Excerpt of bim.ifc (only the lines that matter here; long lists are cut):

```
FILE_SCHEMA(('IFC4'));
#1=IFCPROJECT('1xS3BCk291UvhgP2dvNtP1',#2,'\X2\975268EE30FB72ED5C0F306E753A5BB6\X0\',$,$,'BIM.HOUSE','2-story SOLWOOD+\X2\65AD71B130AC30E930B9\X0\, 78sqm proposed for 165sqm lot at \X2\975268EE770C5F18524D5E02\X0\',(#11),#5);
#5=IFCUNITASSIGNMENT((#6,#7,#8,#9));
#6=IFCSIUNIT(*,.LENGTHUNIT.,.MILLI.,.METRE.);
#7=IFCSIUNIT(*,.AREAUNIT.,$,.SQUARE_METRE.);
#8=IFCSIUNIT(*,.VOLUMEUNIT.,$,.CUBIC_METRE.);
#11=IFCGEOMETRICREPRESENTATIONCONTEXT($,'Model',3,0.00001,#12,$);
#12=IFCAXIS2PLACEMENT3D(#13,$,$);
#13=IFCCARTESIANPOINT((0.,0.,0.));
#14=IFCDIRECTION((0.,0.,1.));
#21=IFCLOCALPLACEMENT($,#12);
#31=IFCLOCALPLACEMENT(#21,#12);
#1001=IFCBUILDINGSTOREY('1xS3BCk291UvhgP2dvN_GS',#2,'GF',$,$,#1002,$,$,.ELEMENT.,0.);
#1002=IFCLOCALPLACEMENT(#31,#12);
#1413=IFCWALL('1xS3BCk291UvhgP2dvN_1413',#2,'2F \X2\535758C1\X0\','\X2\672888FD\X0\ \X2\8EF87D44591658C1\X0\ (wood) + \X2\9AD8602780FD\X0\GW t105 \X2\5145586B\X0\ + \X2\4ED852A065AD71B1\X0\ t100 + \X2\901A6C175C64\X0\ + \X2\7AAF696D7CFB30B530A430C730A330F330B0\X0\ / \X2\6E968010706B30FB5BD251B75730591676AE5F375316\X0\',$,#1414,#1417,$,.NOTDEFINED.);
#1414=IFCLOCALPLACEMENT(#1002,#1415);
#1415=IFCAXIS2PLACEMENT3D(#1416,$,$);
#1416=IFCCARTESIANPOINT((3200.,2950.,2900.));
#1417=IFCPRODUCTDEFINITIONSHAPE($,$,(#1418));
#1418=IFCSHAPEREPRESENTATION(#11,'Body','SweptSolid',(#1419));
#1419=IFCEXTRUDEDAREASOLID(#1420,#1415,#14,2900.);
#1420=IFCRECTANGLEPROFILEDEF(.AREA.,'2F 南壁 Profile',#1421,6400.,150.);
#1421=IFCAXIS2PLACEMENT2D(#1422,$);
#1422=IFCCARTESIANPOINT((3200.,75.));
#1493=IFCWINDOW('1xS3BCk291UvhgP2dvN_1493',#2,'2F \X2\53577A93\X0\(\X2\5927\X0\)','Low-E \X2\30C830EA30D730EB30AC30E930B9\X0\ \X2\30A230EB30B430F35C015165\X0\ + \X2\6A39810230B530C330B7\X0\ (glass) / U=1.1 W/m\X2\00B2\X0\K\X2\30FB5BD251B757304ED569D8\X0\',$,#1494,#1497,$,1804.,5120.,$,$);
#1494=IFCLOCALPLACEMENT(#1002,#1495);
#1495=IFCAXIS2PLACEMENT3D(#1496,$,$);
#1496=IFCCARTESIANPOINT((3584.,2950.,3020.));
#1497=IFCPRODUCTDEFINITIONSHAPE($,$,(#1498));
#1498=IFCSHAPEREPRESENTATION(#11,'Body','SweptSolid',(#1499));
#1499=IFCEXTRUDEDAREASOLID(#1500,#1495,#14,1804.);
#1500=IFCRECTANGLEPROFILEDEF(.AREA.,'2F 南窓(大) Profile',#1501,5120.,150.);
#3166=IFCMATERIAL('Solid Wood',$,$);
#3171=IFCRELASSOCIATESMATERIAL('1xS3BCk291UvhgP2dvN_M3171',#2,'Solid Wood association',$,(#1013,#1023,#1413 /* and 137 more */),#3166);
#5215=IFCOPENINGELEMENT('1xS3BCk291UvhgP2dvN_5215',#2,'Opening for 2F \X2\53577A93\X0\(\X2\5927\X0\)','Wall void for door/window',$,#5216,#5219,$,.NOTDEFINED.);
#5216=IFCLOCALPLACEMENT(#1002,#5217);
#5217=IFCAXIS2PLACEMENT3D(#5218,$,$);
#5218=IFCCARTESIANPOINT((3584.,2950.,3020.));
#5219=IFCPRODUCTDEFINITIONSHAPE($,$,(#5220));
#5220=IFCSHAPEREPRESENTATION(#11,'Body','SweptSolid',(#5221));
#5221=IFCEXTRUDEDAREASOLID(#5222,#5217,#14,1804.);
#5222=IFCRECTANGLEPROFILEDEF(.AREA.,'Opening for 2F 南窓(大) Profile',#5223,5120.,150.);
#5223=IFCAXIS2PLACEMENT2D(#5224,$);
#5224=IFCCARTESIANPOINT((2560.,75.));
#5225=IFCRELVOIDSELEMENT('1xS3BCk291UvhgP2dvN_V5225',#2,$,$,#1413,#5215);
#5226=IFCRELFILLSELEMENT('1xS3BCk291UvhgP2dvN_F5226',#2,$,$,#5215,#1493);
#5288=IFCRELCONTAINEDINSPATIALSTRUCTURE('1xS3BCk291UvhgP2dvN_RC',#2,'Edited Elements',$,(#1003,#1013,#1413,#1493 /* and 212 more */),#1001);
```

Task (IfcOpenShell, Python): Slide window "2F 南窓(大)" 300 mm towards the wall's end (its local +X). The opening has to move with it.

```python
import ifcopenshell
import ifcopenshell.api.geometry
import ifcopenshell.util.placement

model = ifcopenshell.open("bim.ifc")

window = model.by_id(1493)
opening = window.FillsVoids[0].RelatingOpeningElement
wall = opening.VoidsElements[0].RelatingBuildingElement

wall_matrix = ifcopenshell.util.placement.get_local_placement(wall.ObjectPlacement)
shift = wall_matrix[:3, 0] * 300.0
before = ifcopenshell.util.placement.get_local_placement(window.ObjectPlacement)[:3, 3].copy()

# The window is not placed relative to its opening, so move both.
for product in (opening, window):
    matrix = ifcopenshell.util.placement.get_local_placement(product.ObjectPlacement)
    matrix[:3, 3] += shift
    ifcopenshell.api.geometry.edit_object_placement(model, product=product, matrix=matrix, is_si=False)

after = ifcopenshell.util.placement.get_local_placement(window.ObjectPlacement)[:3, 3]
print("window moved by", (after - before).round(3) + 0.0)

model.write("bim-out.ifc")
```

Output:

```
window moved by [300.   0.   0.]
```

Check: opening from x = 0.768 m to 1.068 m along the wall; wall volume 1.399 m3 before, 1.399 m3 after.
